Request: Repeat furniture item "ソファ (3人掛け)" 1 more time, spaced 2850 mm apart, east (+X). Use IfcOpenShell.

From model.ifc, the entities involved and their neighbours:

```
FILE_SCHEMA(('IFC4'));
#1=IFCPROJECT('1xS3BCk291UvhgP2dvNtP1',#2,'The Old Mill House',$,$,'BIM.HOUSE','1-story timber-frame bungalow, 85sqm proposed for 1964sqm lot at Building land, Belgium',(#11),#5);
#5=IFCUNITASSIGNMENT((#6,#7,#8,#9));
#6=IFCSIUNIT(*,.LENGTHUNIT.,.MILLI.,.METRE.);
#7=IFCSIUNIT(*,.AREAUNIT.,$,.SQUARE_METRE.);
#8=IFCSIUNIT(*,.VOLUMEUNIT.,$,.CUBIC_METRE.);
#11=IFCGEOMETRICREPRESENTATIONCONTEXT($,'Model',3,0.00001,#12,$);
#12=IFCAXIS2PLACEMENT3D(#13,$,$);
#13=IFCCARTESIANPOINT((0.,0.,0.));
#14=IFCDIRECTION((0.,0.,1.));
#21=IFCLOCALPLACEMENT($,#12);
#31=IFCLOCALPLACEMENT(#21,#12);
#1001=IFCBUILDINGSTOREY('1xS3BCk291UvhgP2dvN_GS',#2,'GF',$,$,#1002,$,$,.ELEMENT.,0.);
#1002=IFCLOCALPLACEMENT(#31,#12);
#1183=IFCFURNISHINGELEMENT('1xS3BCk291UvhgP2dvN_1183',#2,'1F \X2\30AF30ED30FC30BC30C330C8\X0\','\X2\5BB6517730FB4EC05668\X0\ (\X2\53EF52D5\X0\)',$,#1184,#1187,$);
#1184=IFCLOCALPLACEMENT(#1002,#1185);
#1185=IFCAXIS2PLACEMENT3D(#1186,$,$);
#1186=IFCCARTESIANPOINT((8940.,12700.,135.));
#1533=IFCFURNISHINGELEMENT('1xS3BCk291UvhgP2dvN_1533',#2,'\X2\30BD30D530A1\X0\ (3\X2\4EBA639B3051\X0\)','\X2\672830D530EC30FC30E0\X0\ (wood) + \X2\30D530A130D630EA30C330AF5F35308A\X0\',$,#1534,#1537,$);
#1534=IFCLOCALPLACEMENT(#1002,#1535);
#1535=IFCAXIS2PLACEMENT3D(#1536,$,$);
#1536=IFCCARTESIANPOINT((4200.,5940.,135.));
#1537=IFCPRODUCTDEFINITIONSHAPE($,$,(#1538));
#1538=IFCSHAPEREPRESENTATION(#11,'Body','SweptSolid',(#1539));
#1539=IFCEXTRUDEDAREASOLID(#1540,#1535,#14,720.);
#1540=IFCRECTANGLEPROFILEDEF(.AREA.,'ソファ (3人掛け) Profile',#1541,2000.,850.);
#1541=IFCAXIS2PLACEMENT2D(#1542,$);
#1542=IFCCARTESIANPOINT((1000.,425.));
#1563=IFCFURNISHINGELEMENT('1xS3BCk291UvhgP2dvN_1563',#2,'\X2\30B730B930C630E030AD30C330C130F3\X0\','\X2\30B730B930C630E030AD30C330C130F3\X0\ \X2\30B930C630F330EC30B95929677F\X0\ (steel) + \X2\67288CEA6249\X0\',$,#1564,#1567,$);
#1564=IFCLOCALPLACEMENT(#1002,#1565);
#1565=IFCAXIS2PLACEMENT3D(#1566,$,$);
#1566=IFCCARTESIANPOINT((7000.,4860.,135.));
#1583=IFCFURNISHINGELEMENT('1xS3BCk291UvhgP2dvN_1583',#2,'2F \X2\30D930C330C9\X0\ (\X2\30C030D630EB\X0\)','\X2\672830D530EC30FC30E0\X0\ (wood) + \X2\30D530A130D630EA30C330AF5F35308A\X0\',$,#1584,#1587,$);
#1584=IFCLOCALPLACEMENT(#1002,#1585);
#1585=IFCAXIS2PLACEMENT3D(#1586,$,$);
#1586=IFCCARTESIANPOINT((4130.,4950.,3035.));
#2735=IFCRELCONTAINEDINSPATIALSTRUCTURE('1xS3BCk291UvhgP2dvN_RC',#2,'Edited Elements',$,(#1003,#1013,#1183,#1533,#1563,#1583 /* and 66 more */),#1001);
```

```python
import numpy as np
import ifcopenshell
import ifcopenshell.api.geometry
import ifcopenshell.api.root
import ifcopenshell.util.element
import ifcopenshell.util.placement
import ifcopenshell.util.unit

model = ifcopenshell.open("model.ifc")
unit_scale = ifcopenshell.util.unit.calculate_unit_scale(model)


def reuse_history(source, copy):
    """copy_class also copies each property set's owner history, people and application; keep the originals."""
    for rel in copy.IsDefinedBy:
        if rel.is_a("IfcRelDefinesByProperties") and (history := rel.RelatingPropertyDefinition.OwnerHistory):
            rel.RelatingPropertyDefinition.OwnerHistory = source.OwnerHistory
            ifcopenshell.util.element.remove_deep2(model, history)


source = model.by_guid("1xS3BCk291UvhgP2dvN_1533")
base = ifcopenshell.util.placement.get_local_placement(source.ObjectPlacement)
step = np.array([1.0, 0.0, 0.0]) * 2.85 / unit_scale

for i in range(1, 2):
    copy = ifcopenshell.api.root.copy_class(model, product=source)
    copy.Representation = ifcopenshell.util.element.copy_deep(
        model, source.Representation, exclude=["IfcGeometricRepresentationContext", "IfcRepresentationMap"]
    )
    reuse_history(source, copy)
    matrix = base.copy()
    matrix[:3, 3] += i * step
    print("added at", matrix[:3, 3].round(3) + 0.0)
    ifcopenshell.api.geometry.edit_object_placement(model, product=copy, matrix=matrix, is_si=False)

model.write("model_edited.ifc")
```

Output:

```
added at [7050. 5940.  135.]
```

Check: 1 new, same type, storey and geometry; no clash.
